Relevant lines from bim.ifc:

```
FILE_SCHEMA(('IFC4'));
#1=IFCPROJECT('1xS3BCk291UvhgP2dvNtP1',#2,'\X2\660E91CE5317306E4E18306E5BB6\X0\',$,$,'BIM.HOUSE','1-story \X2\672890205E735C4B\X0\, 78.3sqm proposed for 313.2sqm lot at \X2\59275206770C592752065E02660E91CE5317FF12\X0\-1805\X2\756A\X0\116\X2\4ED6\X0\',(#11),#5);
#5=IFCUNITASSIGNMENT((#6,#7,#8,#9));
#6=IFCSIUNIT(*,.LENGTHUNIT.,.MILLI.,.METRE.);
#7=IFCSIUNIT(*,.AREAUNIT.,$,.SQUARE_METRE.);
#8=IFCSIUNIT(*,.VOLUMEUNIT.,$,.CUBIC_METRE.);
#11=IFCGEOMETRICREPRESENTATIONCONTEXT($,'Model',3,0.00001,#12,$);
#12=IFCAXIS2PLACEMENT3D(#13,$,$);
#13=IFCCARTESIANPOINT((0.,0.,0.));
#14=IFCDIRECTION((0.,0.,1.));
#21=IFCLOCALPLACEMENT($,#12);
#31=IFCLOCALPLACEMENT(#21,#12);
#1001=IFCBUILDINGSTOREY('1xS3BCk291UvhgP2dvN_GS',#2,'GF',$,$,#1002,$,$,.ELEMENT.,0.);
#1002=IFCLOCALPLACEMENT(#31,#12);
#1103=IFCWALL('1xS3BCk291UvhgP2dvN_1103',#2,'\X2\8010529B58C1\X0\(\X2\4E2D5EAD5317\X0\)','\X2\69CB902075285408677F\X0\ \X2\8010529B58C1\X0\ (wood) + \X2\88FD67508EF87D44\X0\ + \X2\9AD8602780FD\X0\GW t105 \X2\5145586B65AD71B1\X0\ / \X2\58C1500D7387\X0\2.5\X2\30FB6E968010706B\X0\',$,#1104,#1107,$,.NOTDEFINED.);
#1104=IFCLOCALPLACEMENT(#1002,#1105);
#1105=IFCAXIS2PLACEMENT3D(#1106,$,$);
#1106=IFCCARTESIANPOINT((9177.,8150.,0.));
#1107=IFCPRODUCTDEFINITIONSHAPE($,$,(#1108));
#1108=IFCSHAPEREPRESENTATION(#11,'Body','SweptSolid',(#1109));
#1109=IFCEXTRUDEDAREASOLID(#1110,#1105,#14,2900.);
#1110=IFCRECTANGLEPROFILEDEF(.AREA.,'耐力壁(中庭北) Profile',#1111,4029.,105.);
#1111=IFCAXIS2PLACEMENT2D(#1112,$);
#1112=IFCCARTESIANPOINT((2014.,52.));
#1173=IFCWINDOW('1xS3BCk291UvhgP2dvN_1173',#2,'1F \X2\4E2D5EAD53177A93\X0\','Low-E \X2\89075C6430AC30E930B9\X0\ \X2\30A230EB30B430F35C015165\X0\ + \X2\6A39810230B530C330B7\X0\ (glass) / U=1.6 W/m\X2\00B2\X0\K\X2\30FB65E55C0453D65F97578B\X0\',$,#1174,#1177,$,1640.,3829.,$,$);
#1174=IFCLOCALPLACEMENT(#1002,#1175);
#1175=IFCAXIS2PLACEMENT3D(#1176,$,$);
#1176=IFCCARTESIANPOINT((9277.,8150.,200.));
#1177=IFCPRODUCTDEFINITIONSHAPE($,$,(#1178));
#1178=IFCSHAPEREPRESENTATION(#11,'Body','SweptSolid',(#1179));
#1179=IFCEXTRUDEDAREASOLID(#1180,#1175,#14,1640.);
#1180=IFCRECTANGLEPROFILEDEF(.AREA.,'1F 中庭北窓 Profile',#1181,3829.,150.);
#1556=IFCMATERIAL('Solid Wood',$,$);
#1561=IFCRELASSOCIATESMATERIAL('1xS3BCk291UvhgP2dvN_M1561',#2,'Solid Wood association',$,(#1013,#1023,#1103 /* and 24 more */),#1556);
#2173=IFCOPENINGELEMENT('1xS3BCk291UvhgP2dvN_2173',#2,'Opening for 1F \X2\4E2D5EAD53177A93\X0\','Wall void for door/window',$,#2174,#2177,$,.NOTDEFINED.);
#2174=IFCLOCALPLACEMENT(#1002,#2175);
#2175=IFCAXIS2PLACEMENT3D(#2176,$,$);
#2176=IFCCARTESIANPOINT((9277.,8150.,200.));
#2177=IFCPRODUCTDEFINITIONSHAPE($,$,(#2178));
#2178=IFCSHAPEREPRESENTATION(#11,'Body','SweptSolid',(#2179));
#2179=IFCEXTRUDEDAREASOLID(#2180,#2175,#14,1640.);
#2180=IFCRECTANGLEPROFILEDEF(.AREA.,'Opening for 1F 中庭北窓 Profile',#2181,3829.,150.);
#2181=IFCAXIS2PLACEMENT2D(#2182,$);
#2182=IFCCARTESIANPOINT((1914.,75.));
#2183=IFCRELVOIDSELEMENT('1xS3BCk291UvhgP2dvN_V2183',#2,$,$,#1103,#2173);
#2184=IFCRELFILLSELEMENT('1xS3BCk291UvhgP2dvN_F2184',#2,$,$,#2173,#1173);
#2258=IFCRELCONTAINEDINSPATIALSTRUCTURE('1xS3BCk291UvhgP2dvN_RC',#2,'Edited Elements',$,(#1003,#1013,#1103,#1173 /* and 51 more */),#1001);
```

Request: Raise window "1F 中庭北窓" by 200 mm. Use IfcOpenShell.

```python
import numpy as np
import ifcopenshell
import ifcopenshell.api.geometry
import ifcopenshell.util.placement
import ifcopenshell.util.unit

model = ifcopenshell.open("bim.ifc")
unit_scale = ifcopenshell.util.unit.calculate_unit_scale(model)

window = model.by_id(1173)
opening = window.FillsVoids[0].RelatingOpeningElement
dz = 0.2 / unit_scale

shift = np.array([0.0, 0.0, dz])
# The window is not placed relative to its opening, so move both.
for product in (opening, window):
    matrix = ifcopenshell.util.placement.get_local_placement(product.ObjectPlacement)
    matrix[:3, 3] += shift
    ifcopenshell.api.geometry.edit_object_placement(model, product=product, matrix=matrix, is_si=False)

print(f"moved by {dz * unit_scale:+.3f} m")

model.write("bim-out.ifc")
```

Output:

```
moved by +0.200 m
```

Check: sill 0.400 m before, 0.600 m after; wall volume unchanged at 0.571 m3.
